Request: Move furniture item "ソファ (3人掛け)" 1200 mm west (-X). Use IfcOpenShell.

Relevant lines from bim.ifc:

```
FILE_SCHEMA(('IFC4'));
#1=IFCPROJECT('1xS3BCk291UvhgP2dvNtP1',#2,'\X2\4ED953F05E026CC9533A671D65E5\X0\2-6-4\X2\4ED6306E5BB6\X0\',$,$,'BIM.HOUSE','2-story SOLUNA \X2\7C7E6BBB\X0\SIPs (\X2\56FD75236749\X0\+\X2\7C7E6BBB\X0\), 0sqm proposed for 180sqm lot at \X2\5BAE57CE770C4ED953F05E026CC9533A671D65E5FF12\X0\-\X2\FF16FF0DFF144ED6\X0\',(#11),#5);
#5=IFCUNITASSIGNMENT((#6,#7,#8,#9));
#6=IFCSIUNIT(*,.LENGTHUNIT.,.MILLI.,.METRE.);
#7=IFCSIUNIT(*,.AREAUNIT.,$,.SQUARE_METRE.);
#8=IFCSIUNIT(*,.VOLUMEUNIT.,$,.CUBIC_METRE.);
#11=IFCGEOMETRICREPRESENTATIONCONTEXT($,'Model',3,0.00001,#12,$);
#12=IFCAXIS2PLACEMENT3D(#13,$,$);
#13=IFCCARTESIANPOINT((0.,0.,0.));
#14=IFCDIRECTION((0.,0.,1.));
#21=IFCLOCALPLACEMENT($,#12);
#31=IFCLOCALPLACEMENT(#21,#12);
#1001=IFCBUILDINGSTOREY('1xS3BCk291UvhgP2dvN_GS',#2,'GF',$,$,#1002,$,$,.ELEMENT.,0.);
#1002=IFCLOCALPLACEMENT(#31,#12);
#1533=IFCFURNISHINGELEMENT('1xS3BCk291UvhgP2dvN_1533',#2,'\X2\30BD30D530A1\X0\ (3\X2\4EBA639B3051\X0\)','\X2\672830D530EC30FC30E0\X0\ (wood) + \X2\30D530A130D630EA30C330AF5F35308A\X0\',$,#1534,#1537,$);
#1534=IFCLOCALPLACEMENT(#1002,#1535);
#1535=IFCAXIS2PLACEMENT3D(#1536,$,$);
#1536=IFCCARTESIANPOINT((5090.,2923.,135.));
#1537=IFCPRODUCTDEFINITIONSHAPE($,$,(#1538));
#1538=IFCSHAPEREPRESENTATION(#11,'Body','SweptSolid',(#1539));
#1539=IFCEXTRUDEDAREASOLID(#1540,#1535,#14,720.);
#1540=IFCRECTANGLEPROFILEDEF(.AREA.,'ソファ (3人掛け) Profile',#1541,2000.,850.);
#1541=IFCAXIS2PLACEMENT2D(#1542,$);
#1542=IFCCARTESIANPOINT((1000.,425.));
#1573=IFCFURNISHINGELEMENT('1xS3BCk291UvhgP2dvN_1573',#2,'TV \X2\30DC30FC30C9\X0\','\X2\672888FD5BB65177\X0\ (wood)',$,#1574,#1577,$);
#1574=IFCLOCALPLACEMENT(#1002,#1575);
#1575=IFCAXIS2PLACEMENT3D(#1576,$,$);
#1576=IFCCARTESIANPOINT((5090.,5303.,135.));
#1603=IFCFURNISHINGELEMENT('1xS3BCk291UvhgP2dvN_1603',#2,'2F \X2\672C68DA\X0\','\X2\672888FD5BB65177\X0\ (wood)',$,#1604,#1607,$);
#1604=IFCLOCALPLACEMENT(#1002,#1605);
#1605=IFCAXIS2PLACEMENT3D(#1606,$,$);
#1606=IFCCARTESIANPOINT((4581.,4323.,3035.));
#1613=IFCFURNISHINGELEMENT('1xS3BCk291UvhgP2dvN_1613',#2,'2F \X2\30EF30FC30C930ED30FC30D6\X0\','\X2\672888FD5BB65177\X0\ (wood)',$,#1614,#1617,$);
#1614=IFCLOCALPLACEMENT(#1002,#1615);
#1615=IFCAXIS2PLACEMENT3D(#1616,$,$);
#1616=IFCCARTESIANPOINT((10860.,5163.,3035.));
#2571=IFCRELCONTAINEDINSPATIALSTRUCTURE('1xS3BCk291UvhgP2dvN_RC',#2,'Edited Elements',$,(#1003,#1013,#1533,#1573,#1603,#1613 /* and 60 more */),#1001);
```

```python
import ifcopenshell
import ifcopenshell.api.geometry
import ifcopenshell.util.placement
import ifcopenshell.util.unit

model = ifcopenshell.open("bim.ifc")
unit_scale = ifcopenshell.util.unit.calculate_unit_scale(model)

item = model.by_id(1533)
matrix = ifcopenshell.util.placement.get_local_placement(item.ObjectPlacement)
matrix[0, 3] -= 1.2 / unit_scale
ifcopenshell.api.geometry.edit_object_placement(model, product=item, matrix=matrix, is_si=False)

print(ifcopenshell.util.placement.get_local_placement(item.ObjectPlacement).round(3) + 0.0)

model.write("bim_updated.ifc")
```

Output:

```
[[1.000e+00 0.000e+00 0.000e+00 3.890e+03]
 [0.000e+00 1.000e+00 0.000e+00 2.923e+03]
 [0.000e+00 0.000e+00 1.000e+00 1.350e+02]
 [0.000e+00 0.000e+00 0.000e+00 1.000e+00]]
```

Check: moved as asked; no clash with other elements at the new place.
